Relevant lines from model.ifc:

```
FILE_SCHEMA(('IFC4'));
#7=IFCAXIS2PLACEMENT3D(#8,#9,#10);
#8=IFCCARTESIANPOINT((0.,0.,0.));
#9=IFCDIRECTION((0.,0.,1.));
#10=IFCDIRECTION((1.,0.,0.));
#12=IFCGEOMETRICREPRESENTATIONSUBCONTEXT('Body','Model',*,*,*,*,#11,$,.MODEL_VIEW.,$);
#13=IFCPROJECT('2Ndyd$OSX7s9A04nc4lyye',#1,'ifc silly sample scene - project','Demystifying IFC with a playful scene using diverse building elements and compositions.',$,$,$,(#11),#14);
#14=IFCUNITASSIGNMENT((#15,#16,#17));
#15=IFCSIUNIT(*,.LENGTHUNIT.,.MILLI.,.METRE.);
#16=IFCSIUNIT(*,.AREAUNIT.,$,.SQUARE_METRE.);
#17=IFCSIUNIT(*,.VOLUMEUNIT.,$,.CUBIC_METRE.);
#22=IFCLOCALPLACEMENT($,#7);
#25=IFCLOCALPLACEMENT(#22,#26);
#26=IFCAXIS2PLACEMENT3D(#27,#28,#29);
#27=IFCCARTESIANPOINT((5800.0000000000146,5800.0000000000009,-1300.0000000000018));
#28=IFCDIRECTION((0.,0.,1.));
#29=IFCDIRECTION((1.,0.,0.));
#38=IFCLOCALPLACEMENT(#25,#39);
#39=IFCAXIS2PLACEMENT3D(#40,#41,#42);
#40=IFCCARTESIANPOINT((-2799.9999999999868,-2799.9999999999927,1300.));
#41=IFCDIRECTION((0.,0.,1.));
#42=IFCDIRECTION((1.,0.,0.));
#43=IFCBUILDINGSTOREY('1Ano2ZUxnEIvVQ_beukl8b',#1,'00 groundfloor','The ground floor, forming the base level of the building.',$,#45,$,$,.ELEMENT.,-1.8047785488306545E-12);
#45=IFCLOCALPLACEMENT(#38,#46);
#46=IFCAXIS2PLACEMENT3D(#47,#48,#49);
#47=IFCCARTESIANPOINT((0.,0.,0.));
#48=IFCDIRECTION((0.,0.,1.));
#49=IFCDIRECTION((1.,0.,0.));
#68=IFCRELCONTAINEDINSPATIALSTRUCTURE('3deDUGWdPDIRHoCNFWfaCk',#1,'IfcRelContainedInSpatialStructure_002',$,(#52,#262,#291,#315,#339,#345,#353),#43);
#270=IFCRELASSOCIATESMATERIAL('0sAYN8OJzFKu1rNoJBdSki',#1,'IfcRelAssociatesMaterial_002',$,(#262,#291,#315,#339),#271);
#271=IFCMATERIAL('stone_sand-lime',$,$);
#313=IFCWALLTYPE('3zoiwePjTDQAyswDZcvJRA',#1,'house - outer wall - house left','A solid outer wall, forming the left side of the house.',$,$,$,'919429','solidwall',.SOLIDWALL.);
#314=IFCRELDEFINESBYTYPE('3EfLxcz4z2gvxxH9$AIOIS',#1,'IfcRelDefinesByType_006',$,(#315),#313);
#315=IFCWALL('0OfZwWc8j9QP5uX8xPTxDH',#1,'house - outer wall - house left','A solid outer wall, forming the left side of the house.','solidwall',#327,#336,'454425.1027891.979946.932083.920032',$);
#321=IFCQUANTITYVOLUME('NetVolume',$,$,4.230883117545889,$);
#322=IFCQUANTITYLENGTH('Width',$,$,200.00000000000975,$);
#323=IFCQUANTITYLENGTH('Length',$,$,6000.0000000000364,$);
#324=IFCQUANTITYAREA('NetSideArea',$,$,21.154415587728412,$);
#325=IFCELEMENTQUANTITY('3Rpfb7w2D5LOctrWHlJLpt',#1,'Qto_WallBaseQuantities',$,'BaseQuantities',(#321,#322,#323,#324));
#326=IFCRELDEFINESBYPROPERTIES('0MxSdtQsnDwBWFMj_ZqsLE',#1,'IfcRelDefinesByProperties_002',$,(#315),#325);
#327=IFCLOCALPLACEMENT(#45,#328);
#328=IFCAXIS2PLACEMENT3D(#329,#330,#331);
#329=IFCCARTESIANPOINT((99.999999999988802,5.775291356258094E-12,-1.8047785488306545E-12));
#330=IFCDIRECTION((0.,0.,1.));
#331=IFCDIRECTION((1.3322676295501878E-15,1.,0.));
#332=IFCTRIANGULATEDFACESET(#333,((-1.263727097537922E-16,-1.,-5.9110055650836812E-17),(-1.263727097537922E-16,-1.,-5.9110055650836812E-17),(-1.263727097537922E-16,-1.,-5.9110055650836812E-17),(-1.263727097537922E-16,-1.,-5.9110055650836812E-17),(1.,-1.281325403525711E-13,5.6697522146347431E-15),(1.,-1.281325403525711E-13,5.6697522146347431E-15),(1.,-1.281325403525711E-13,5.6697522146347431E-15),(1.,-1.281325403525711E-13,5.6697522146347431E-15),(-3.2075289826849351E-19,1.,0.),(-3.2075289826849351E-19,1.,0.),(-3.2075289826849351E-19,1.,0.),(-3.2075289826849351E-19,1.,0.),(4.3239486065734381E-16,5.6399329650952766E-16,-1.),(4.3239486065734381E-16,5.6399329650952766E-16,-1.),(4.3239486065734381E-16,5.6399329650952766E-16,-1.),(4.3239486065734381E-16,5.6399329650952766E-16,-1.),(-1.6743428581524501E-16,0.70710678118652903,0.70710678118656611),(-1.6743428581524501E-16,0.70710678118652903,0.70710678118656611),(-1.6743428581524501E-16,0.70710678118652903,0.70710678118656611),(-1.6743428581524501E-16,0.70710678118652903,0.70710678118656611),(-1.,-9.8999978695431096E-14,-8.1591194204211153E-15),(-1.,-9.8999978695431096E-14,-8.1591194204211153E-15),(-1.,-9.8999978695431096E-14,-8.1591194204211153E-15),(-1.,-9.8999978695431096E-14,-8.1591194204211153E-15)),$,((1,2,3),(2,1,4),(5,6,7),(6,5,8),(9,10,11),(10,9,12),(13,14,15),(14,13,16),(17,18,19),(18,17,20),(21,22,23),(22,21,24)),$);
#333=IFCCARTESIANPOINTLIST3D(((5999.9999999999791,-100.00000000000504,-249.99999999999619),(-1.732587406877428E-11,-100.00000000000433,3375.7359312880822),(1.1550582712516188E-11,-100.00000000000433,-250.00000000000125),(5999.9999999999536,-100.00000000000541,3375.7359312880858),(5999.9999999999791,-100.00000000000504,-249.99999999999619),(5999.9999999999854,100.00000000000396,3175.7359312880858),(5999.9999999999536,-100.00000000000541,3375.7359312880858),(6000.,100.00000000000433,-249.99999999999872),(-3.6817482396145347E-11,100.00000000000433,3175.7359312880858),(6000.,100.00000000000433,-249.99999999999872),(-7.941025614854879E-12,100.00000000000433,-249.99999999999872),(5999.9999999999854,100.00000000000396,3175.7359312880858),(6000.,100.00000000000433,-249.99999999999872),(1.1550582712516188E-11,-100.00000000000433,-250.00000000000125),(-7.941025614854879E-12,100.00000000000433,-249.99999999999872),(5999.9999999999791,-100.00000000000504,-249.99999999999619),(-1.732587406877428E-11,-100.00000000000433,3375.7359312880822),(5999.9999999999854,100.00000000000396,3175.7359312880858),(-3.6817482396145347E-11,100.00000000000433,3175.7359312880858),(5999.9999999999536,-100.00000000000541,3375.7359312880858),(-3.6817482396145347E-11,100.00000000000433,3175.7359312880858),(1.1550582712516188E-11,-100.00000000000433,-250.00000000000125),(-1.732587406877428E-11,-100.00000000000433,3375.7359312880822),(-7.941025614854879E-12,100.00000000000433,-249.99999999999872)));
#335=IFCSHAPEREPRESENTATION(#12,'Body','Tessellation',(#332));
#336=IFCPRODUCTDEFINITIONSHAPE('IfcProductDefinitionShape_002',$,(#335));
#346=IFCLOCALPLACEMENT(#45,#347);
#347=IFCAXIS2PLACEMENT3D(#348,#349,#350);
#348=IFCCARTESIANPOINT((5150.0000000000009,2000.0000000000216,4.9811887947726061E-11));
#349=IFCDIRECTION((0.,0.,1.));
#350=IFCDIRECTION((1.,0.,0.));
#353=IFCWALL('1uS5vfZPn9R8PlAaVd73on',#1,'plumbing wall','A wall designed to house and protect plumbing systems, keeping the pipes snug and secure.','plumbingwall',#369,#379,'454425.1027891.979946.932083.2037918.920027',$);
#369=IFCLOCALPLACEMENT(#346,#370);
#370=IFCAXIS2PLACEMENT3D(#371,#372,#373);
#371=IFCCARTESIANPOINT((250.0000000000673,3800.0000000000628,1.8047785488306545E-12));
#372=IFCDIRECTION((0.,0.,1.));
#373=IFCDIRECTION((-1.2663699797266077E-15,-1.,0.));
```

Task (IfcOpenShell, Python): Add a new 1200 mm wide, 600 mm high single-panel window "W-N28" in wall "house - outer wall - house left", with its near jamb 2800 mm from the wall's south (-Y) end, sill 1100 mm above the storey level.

```python
import numpy as np
import ifcopenshell
import ifcopenshell.api.feature
import ifcopenshell.api.geometry
import ifcopenshell.api.pset
import ifcopenshell.api.root
import ifcopenshell.api.spatial
import ifcopenshell.geom
import ifcopenshell.util.element
import ifcopenshell.util.placement
import ifcopenshell.util.representation
import ifcopenshell.util.shape
import ifcopenshell.util.unit

model = ifcopenshell.open("model.ifc")
unit_scale = ifcopenshell.util.unit.calculate_unit_scale(model)
area_scale = ifcopenshell.util.unit.calculate_unit_scale(model, "AREAUNIT")
volume_scale = ifcopenshell.util.unit.calculate_unit_scale(model, "VOLUMEUNIT")
settings = ifcopenshell.geom.settings()


def volume(element):
    """Net volume in cubic metres, openings subtracted."""
    shape = ifcopenshell.geom.create_shape(settings, element)
    return ifcopenshell.util.shape.get_volume(shape.geometry)


wall = model.by_guid("0OfZwWc8j9QP5uX8xPTxDH")
storey = ifcopenshell.util.element.get_container(wall, ifc_class="IfcBuildingStorey")
context = ifcopenshell.util.representation.get_context(model, "Model", "Body", "MODEL_VIEW")
before = volume(wall)

width, height, from_end, sill = 1.2, 0.6, 2.8, 1.1  # metres

# The wall runs along its own X axis, and the end named is its -X end.
wall_shape = ifcopenshell.geom.create_shape(settings, wall)
x, y, z = ifcopenshell.util.shape.get_vertices(wall_shape.geometry).T
start = x.min() + from_end
face, thickness = float(y.min()), float(y.max() - y.min())
wall_matrix = ifcopenshell.util.placement.get_local_placement(wall.ObjectPlacement)
level = ifcopenshell.util.placement.get_local_placement(storey.ObjectPlacement)[2, 3]


def in_wall(x, y):
    """Placement at x, y metres in the wall's axes, at sill height."""
    matrix = wall_matrix.copy()
    matrix[:, 3] = wall_matrix @ np.array([x / unit_scale, y / unit_scale, 0.0, 1.0])
    matrix[2, 3] = level + sill / unit_scale
    return matrix


# Opening: a box that overshoots both wall faces by 50 mm.
opening = ifcopenshell.api.root.create_entity(model, ifc_class="IfcOpeningElement", predefined_type="OPENING")
box = ifcopenshell.api.geometry.add_wall_representation(
    model, context=context, length=width, height=height, thickness=thickness + 0.1
)
ifcopenshell.api.geometry.assign_representation(model, product=opening, representation=box)
ifcopenshell.api.geometry.edit_object_placement(model, product=opening, matrix=in_wall(start, face - 0.05), is_si=False)
ifcopenshell.api.feature.add_feature(model, feature=opening, element=wall)

window = ifcopenshell.api.root.create_entity(model, ifc_class="IfcWindow", name="W-N28", predefined_type="WINDOW")
window.OverallWidth, window.OverallHeight = width / unit_scale, height / unit_scale
window.PartitioningType = "SINGLE_PANEL"
body = ifcopenshell.api.geometry.add_window_representation(
    model,
    context=context,
    overall_width=window.OverallWidth,
    overall_height=window.OverallHeight,
    partition_type="SINGLE_PANEL",
)
ifcopenshell.api.geometry.assign_representation(model, product=window, representation=body)
ifcopenshell.api.spatial.assign_container(model, products=[window], relating_structure=storey)
ifcopenshell.api.feature.add_filling(model, opening=opening, element=window)

# Centre the window in the wall's thickness.
ifcopenshell.api.geometry.edit_object_placement(model, product=window, matrix=in_wall(start, face), is_si=False)
window_shape = ifcopenshell.geom.create_shape(settings, window)
depth = ifcopenshell.util.shape.get_vertices(window_shape.geometry)[:, 1]
offset = face + thickness / 2 - (depth.min() + depth.max()) / 2
ifcopenshell.api.geometry.edit_object_placement(model, product=window, matrix=in_wall(start, offset), is_si=False)

after = volume(wall)

# Update the wall's stored quantities.
qto = model.by_id(ifcopenshell.util.element.get_pset(wall, "Qto_WallBaseQuantities", should_inherit=False)["id"])
ifcopenshell.api.pset.edit_qto(model, qto=qto, properties={
    "NetVolume": after / volume_scale,
    "NetSideArea": after / thickness / area_scale,
})

print(f"wall volume {before:.3f} -> {after:.3f} m3")

model.write("model_edited.ifc")
```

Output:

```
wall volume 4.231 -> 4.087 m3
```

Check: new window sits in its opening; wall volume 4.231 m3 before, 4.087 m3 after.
